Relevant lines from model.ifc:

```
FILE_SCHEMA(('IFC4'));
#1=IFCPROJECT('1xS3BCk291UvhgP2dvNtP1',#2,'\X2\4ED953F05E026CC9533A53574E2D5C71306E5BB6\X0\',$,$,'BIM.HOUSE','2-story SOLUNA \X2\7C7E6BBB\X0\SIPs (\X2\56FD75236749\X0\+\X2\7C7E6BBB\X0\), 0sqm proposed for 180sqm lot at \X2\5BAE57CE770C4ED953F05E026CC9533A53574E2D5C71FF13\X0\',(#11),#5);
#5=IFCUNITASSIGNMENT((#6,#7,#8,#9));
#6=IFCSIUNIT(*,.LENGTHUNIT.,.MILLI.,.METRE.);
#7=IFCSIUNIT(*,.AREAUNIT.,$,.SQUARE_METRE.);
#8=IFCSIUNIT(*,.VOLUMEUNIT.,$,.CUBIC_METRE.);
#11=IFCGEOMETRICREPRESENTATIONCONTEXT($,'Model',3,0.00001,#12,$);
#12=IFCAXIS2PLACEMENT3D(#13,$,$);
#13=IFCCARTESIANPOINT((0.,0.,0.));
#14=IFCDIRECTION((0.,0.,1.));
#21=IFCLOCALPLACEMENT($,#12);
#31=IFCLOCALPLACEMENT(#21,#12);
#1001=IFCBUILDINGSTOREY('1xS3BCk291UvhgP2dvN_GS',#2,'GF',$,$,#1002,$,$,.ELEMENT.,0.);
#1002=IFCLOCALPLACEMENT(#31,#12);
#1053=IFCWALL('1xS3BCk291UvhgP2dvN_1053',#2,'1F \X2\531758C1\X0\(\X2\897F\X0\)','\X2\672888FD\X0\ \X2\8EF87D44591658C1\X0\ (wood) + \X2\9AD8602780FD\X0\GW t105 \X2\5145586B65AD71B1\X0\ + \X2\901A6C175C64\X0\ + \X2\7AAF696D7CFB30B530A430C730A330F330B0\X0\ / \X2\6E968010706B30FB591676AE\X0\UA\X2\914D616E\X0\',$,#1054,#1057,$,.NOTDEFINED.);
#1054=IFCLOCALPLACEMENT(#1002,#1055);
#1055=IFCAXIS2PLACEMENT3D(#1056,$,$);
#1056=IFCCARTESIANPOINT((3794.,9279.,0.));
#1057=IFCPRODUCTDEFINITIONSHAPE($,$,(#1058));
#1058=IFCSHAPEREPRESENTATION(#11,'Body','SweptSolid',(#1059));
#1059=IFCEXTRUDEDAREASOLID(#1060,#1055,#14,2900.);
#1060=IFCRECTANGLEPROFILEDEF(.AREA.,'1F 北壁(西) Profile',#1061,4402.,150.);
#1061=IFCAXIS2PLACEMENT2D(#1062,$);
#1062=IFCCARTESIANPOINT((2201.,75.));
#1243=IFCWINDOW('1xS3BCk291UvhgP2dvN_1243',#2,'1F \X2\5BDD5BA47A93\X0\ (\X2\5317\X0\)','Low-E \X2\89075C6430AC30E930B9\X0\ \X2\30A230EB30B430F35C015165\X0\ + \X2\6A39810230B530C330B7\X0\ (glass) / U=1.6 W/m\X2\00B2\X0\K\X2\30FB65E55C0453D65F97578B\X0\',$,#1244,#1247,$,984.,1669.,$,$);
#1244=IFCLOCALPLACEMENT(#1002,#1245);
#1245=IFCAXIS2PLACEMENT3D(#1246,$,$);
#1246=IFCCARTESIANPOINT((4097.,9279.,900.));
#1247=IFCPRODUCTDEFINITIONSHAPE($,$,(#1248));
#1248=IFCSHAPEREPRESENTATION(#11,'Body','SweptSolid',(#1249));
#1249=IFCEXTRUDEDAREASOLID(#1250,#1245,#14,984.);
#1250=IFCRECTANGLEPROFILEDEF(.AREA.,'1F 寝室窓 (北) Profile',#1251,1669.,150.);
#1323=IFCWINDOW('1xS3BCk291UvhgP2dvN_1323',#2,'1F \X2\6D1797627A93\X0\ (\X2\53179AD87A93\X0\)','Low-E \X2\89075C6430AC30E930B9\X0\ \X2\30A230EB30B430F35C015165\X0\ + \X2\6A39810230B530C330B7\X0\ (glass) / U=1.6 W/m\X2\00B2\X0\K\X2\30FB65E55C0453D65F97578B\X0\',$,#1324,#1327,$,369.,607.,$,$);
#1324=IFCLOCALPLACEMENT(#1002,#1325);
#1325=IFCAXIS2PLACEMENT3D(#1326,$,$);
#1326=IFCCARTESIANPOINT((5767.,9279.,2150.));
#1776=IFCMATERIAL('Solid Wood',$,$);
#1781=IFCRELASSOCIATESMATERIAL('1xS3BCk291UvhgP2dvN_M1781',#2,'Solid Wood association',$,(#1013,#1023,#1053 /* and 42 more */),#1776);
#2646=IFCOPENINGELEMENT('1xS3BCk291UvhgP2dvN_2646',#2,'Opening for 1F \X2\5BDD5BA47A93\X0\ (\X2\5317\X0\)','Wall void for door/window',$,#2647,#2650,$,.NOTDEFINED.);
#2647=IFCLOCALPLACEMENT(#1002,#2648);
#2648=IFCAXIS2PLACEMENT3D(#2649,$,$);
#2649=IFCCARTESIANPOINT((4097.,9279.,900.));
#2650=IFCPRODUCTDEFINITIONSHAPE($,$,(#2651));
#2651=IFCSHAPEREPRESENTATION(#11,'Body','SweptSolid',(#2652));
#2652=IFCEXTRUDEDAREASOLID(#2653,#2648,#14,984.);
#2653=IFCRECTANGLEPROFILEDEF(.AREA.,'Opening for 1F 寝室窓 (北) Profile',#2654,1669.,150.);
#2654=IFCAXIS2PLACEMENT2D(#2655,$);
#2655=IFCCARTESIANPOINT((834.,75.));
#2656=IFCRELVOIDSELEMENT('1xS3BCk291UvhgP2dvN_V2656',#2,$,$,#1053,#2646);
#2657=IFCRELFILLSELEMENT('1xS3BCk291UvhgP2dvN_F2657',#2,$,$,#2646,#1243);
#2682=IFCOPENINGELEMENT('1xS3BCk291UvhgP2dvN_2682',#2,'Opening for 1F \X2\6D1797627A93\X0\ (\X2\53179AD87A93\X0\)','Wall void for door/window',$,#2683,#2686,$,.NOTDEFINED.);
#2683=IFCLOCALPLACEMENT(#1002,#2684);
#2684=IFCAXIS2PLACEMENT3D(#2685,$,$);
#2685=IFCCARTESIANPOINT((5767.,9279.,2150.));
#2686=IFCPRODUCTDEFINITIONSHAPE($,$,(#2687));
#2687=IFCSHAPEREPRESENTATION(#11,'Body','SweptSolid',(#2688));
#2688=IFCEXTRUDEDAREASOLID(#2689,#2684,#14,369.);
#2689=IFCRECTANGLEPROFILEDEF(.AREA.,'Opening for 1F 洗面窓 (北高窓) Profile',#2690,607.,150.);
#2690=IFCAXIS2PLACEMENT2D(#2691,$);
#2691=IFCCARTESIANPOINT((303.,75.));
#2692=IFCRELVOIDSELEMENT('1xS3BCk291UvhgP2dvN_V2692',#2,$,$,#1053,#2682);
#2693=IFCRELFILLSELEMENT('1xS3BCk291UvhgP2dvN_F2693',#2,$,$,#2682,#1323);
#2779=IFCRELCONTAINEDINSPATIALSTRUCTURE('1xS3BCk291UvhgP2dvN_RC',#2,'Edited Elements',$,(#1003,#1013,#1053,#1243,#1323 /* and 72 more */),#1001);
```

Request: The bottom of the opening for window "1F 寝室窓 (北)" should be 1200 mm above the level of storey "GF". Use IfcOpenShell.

```python
import numpy as np
import ifcopenshell
import ifcopenshell.api.geometry
import ifcopenshell.geom
import ifcopenshell.util.element
import ifcopenshell.util.placement
import ifcopenshell.util.shape
import ifcopenshell.util.unit

model = ifcopenshell.open("model.ifc")
unit_scale = ifcopenshell.util.unit.calculate_unit_scale(model)

window = model.by_id(1243)
opening = window.FillsVoids[0].RelatingOpeningElement
storey = ifcopenshell.util.element.get_container(window, ifc_class="IfcBuildingStorey")
level = ifcopenshell.util.placement.get_local_placement(storey.ObjectPlacement)[2, 3]

# The opening's origin need not be at the sill, so measure its lowest point.
shape = ifcopenshell.geom.create_shape(ifcopenshell.geom.settings(), opening)
bottom = ifcopenshell.util.shape.get_shape_bottom_elevation(shape, shape.geometry) / unit_scale
dz = level + 1.2 / unit_scale - bottom

shift = np.array([0.0, 0.0, dz])
# The window is not placed relative to its opening, so move both.
for product in (opening, window):
    matrix = ifcopenshell.util.placement.get_local_placement(product.ObjectPlacement)
    matrix[:3, 3] += shift
    ifcopenshell.api.geometry.edit_object_placement(model, product=product, matrix=matrix, is_si=False)

print(f"moved by {dz * unit_scale:+.3f} m")

model.write("model_v2.ifc")
```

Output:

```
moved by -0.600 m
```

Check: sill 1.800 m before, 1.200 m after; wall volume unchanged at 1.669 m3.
